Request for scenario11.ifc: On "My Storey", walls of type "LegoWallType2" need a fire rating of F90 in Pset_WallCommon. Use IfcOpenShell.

First a look at what the model holds.

```python
import ifcopenshell
import ifcopenshell.util.element

model = ifcopenshell.open("scenario11.ifc")
print(model.schema)
storey = next(s for s in model.by_type("IfcBuildingStorey") if s.Name == "My Storey")
walls = [e for e in ifcopenshell.util.element.get_decomposition(storey) if e.is_a("IfcWall")]
seen = {}
for e in walls:
    element_type = ifcopenshell.util.element.get_type(e)
    key = (element_type.Name if element_type != e and element_type else None, ifcopenshell.util.element.get_pset(e, "Pset_WallCommon", "FireRating"))
    seen[key] = seen.get(key, 0) + 1
for (name, value), count in sorted(seen.items(), key=str):
    print(count, "x", name, "|", value)
```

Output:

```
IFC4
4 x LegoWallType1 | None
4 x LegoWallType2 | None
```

```python
import ifcopenshell
import ifcopenshell.api.pset
import ifcopenshell.util.element

model = ifcopenshell.open("scenario11.ifc")

storey = next(s for s in model.by_type("IfcBuildingStorey") if s.Name == "My Storey")
walls = [e for e in ifcopenshell.util.element.get_decomposition(storey) if e.is_a("IfcWall")]

count = 0
for e in walls:
    element_type = ifcopenshell.util.element.get_type(e)
    if element_type in (None, e) or element_type.Name != "LegoWallType2":
        continue
    # add_pset returns the element's existing set when there is one.
    pset = ifcopenshell.api.pset.add_pset(model, product=e, name="Pset_WallCommon")
    ifcopenshell.api.pset.edit_pset(model, pset=pset, properties={"FireRating": "F90"})
    count += 1

print(count, "walls updated")

model.write("scenario11_edited.ifc")
```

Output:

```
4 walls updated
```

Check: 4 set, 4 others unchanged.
